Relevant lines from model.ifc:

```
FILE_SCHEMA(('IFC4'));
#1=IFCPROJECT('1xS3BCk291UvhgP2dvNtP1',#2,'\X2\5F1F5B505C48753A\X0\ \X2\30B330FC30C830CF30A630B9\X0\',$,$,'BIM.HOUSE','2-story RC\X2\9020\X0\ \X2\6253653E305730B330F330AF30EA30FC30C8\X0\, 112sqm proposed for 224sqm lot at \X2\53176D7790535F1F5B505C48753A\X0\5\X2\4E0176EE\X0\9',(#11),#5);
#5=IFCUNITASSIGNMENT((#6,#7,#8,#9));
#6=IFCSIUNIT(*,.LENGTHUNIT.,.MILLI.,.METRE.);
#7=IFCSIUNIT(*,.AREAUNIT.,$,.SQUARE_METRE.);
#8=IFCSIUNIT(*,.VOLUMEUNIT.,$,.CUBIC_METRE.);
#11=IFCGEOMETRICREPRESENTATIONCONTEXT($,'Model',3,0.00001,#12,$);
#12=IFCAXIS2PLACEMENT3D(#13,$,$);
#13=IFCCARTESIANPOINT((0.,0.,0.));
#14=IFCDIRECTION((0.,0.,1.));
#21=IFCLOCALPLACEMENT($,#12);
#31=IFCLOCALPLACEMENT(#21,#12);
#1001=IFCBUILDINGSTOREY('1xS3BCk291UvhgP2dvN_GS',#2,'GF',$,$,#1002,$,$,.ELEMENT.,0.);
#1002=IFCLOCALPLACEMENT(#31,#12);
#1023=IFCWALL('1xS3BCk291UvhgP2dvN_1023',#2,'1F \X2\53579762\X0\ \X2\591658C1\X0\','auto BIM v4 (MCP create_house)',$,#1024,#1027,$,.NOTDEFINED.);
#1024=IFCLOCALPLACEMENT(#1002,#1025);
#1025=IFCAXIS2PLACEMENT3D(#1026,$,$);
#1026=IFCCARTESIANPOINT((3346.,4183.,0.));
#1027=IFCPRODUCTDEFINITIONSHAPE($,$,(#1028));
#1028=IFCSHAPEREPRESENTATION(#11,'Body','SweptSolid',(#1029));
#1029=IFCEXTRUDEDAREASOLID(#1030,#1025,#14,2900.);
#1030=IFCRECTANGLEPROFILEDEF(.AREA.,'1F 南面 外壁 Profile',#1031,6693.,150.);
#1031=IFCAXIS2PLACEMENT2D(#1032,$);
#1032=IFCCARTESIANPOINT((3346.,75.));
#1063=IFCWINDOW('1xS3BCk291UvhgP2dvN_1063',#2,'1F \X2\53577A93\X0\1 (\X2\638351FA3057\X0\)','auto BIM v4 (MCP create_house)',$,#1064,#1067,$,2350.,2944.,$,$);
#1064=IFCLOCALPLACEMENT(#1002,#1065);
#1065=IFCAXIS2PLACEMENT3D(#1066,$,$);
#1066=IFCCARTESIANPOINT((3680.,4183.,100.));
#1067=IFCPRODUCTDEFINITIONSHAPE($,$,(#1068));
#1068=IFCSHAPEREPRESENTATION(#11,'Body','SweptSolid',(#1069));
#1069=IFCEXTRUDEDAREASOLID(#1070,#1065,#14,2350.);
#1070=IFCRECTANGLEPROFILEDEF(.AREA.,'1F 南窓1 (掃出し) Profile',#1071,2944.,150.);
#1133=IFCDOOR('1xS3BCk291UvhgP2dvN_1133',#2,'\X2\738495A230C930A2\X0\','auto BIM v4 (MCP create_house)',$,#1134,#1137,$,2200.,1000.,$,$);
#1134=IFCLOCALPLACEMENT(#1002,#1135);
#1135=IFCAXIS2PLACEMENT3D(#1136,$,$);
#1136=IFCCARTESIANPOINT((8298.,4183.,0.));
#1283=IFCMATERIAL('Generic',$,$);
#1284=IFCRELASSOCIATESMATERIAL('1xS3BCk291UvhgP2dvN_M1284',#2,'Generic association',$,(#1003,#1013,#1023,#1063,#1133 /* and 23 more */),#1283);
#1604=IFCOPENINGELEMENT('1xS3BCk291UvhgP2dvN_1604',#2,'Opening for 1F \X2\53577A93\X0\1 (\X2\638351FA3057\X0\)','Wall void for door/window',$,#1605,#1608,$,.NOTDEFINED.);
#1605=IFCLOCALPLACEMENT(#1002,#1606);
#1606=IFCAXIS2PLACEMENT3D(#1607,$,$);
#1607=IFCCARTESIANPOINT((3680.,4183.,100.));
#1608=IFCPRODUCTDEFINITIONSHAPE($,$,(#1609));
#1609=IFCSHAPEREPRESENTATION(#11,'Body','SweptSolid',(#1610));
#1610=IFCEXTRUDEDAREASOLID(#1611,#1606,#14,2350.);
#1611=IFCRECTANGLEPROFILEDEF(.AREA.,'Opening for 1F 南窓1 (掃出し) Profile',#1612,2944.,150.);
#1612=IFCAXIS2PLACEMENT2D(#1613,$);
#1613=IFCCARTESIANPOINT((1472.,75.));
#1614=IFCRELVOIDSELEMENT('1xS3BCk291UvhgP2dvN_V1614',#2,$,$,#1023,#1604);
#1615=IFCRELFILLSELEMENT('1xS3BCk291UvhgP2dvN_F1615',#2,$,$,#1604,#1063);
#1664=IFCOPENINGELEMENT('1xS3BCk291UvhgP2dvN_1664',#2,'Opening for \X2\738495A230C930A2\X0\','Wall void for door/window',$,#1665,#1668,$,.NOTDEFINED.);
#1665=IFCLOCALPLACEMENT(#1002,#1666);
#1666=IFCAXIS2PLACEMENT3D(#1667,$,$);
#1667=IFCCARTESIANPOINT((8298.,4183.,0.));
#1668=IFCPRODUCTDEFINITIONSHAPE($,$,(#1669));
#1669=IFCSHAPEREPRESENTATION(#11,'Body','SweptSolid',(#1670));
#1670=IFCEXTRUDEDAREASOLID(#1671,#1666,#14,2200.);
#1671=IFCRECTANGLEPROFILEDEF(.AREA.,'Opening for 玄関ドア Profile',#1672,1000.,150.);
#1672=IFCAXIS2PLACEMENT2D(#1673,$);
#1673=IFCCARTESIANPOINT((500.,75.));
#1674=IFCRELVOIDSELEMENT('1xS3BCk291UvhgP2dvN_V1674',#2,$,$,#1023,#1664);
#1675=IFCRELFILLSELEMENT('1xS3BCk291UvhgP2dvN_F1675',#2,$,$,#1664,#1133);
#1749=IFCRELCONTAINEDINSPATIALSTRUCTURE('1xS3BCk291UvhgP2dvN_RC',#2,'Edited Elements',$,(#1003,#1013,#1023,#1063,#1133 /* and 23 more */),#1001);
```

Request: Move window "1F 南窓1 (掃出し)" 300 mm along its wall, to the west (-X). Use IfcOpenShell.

```python
import ifcopenshell
import ifcopenshell.api.geometry
import ifcopenshell.util.placement
import ifcopenshell.util.unit

model = ifcopenshell.open("model.ifc")
unit_scale = ifcopenshell.util.unit.calculate_unit_scale(model)

window = model.by_guid("1xS3BCk291UvhgP2dvN_1063")
opening = window.FillsVoids[0].RelatingOpeningElement
wall = opening.VoidsElements[0].RelatingBuildingElement

wall_matrix = ifcopenshell.util.placement.get_local_placement(wall.ObjectPlacement)
shift = wall_matrix[:3, 0] * -0.3 / unit_scale
before = ifcopenshell.util.placement.get_local_placement(window.ObjectPlacement)[:3, 3].copy()

# The window is not placed relative to its opening, so move both.
for product in (opening, window):
    matrix = ifcopenshell.util.placement.get_local_placement(product.ObjectPlacement)
    matrix[:3, 3] += shift
    ifcopenshell.api.geometry.edit_object_placement(model, product=product, matrix=matrix, is_si=False)

after = ifcopenshell.util.placement.get_local_placement(window.ObjectPlacement)[:3, 3]
print("window moved by", (after - before).round(3) + 0.0)

model.write("model_v2.ifc")
```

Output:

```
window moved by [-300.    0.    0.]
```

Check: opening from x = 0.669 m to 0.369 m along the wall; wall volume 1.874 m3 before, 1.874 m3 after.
